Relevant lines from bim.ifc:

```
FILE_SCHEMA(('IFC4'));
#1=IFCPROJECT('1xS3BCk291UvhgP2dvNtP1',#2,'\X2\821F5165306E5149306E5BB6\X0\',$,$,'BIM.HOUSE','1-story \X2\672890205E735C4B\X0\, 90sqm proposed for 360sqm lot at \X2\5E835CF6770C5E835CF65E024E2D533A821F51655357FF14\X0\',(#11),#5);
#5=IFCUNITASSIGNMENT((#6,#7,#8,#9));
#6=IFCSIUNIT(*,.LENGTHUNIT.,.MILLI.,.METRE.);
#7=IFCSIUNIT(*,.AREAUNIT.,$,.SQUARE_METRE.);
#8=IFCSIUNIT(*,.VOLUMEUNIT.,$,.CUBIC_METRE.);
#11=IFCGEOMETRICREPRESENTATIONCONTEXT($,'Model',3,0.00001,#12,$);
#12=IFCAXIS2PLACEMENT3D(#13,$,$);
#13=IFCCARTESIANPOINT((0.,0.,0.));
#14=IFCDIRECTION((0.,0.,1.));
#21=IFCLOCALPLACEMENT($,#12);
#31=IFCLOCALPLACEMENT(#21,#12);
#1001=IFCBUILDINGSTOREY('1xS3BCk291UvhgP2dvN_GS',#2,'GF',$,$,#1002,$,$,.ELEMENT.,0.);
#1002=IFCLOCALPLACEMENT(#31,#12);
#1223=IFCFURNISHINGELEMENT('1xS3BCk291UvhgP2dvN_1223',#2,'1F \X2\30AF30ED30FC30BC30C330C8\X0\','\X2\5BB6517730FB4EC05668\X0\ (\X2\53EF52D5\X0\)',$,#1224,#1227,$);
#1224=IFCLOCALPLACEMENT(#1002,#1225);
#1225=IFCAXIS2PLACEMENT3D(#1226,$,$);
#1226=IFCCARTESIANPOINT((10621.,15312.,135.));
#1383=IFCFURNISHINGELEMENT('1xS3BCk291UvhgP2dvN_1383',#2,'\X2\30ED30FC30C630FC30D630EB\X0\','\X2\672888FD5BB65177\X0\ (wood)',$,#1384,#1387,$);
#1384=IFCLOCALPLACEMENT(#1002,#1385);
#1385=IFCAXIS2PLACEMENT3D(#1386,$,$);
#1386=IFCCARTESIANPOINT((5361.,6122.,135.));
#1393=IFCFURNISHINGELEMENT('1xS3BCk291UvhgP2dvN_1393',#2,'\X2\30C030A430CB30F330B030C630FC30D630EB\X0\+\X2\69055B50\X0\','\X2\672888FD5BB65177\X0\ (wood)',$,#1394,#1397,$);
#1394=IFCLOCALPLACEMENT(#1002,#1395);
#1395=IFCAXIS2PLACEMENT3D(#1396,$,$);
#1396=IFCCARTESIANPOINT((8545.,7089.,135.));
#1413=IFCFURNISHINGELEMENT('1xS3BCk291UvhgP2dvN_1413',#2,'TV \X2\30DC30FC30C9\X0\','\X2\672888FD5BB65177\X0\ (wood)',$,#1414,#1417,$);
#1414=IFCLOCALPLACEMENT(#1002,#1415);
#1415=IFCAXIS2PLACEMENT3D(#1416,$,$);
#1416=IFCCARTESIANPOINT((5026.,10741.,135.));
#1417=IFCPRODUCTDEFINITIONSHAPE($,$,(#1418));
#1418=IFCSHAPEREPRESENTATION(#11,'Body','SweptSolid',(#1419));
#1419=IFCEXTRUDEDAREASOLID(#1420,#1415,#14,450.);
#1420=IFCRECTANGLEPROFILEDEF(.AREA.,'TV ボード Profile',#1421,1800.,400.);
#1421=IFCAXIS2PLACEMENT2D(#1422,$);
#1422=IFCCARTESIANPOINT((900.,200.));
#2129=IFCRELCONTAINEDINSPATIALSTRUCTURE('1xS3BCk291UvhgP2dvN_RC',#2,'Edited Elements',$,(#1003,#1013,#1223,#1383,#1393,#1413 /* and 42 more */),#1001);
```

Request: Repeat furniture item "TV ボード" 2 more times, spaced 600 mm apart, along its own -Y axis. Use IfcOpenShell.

```python
import ifcopenshell
import ifcopenshell.api.geometry
import ifcopenshell.api.root
import ifcopenshell.util.element
import ifcopenshell.util.placement

model = ifcopenshell.open("bim.ifc")


def reuse_history(source, copy):
    """copy_class also copies each property set's owner history, people and application; keep the originals."""
    for rel in copy.IsDefinedBy:
        if rel.is_a("IfcRelDefinesByProperties") and (history := rel.RelatingPropertyDefinition.OwnerHistory):
            rel.RelatingPropertyDefinition.OwnerHistory = source.OwnerHistory
            ifcopenshell.util.element.remove_deep2(model, history)


source = model.by_guid("1xS3BCk291UvhgP2dvN_1413")
base = ifcopenshell.util.placement.get_local_placement(source.ObjectPlacement)
step = -base[:3, 1] * 600.0

for i in range(1, 3):
    copy = ifcopenshell.api.root.copy_class(model, product=source)
    copy.Representation = ifcopenshell.util.element.copy_deep(
        model, source.Representation, exclude=["IfcGeometricRepresentationContext", "IfcRepresentationMap"]
    )
    reuse_history(source, copy)
    matrix = base.copy()
    matrix[:3, 3] += i * step
    print("added at", matrix[:3, 3].round(3) + 0.0)
    ifcopenshell.api.geometry.edit_object_placement(model, product=copy, matrix=matrix, is_si=False)

model.write("bim_edited.ifc")
```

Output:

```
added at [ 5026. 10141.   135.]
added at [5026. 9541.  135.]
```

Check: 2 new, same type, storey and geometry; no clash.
